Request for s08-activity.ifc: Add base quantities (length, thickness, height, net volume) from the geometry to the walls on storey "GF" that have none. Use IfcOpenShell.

First a look at what the model holds.

```python
import ifcopenshell
import ifcopenshell.util.element
import ifcopenshell.util.unit

model = ifcopenshell.open("s08-activity.ifc")
print(model.schema)
for unit_type in ("LENGTHUNIT", "AREAUNIT", "VOLUMEUNIT"):
    print(unit_type, ifcopenshell.util.unit.calculate_unit_scale(model, unit_type))
storey = next(s for s in model.by_type("IfcBuildingStorey") if s.Name == "GF")
walls = [e for e in ifcopenshell.util.element.get_decomposition(storey) if e.is_a("IfcWall")]
for e in sorted(walls, key=lambda e: e.id()):
    print(e.id(), e.is_a(), e.Name, list(ifcopenshell.util.element.get_psets(e, qtos_only=True)), sep=" | ")
```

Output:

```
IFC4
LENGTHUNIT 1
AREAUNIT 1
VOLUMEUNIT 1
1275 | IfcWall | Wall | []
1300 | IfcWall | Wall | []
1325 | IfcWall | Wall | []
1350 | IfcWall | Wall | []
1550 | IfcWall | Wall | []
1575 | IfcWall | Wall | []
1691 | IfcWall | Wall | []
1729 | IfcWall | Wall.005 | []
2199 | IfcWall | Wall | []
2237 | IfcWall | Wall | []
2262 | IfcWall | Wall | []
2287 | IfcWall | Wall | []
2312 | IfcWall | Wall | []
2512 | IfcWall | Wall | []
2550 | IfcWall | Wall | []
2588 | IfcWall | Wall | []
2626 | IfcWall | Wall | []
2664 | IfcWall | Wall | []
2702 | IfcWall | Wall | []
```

```python
import ifcopenshell
import ifcopenshell.api.pset
import ifcopenshell.geom
import ifcopenshell.util.element
import ifcopenshell.util.shape
import ifcopenshell.util.unit

model = ifcopenshell.open("s08-activity.ifc")
unit_scale = ifcopenshell.util.unit.calculate_unit_scale(model)
volume_scale = ifcopenshell.util.unit.calculate_unit_scale(model, "VOLUMEUNIT")
settings = ifcopenshell.geom.settings()

storey = next(s for s in model.by_type("IfcBuildingStorey") if s.Name == "GF")
walls = [e for e in ifcopenshell.util.element.get_decomposition(storey) if e.is_a("IfcWall")]

for e in sorted(walls, key=lambda e: e.id()):
    if ifcopenshell.util.element.get_psets(e, qtos_only=True, should_inherit=False):
        continue
    # Geometry comes back in metres, in the element's own axes.
    shape = ifcopenshell.geom.create_shape(settings, e)
    values = {
        "Length": ifcopenshell.util.shape.get_x(shape.geometry) / unit_scale,
        "Width": ifcopenshell.util.shape.get_y(shape.geometry) / unit_scale,
        "Height": ifcopenshell.util.shape.get_z(shape.geometry) / unit_scale,
        "NetVolume": ifcopenshell.util.shape.get_volume(shape.geometry) / volume_scale,
    }
    qto = ifcopenshell.api.pset.add_qto(model, product=e, name="Qto_WallBaseQuantities")
    ifcopenshell.api.pset.edit_qto(model, qto=qto, properties=values)
    print(e.id(), {k: round(v, 3) for k, v in values.items()})

model.write("s08-activity_updated.ifc")
```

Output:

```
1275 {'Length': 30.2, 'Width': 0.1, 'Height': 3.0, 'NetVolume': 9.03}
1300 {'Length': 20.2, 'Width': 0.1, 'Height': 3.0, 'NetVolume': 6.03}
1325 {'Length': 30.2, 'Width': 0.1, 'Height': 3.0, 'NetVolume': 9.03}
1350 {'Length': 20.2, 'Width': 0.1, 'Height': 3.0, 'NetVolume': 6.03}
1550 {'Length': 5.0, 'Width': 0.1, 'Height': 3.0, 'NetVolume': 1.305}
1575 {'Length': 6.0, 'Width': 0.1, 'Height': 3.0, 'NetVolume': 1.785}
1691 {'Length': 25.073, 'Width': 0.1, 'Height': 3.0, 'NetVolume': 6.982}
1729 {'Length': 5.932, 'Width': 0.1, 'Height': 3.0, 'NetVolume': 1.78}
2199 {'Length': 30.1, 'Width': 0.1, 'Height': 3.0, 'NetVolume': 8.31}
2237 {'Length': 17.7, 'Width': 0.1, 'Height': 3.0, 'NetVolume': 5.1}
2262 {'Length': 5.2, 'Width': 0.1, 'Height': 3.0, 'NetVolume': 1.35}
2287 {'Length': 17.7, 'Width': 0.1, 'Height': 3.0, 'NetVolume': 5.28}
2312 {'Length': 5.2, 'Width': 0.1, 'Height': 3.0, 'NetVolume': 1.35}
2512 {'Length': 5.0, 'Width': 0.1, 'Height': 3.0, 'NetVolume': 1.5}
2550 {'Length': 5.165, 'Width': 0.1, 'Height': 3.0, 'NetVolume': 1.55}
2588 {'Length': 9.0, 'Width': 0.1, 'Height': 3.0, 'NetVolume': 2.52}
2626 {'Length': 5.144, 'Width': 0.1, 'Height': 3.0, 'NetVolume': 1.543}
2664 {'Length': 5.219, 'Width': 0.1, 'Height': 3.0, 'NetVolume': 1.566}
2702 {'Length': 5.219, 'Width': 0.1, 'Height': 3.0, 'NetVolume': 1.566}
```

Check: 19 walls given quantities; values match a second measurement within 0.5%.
